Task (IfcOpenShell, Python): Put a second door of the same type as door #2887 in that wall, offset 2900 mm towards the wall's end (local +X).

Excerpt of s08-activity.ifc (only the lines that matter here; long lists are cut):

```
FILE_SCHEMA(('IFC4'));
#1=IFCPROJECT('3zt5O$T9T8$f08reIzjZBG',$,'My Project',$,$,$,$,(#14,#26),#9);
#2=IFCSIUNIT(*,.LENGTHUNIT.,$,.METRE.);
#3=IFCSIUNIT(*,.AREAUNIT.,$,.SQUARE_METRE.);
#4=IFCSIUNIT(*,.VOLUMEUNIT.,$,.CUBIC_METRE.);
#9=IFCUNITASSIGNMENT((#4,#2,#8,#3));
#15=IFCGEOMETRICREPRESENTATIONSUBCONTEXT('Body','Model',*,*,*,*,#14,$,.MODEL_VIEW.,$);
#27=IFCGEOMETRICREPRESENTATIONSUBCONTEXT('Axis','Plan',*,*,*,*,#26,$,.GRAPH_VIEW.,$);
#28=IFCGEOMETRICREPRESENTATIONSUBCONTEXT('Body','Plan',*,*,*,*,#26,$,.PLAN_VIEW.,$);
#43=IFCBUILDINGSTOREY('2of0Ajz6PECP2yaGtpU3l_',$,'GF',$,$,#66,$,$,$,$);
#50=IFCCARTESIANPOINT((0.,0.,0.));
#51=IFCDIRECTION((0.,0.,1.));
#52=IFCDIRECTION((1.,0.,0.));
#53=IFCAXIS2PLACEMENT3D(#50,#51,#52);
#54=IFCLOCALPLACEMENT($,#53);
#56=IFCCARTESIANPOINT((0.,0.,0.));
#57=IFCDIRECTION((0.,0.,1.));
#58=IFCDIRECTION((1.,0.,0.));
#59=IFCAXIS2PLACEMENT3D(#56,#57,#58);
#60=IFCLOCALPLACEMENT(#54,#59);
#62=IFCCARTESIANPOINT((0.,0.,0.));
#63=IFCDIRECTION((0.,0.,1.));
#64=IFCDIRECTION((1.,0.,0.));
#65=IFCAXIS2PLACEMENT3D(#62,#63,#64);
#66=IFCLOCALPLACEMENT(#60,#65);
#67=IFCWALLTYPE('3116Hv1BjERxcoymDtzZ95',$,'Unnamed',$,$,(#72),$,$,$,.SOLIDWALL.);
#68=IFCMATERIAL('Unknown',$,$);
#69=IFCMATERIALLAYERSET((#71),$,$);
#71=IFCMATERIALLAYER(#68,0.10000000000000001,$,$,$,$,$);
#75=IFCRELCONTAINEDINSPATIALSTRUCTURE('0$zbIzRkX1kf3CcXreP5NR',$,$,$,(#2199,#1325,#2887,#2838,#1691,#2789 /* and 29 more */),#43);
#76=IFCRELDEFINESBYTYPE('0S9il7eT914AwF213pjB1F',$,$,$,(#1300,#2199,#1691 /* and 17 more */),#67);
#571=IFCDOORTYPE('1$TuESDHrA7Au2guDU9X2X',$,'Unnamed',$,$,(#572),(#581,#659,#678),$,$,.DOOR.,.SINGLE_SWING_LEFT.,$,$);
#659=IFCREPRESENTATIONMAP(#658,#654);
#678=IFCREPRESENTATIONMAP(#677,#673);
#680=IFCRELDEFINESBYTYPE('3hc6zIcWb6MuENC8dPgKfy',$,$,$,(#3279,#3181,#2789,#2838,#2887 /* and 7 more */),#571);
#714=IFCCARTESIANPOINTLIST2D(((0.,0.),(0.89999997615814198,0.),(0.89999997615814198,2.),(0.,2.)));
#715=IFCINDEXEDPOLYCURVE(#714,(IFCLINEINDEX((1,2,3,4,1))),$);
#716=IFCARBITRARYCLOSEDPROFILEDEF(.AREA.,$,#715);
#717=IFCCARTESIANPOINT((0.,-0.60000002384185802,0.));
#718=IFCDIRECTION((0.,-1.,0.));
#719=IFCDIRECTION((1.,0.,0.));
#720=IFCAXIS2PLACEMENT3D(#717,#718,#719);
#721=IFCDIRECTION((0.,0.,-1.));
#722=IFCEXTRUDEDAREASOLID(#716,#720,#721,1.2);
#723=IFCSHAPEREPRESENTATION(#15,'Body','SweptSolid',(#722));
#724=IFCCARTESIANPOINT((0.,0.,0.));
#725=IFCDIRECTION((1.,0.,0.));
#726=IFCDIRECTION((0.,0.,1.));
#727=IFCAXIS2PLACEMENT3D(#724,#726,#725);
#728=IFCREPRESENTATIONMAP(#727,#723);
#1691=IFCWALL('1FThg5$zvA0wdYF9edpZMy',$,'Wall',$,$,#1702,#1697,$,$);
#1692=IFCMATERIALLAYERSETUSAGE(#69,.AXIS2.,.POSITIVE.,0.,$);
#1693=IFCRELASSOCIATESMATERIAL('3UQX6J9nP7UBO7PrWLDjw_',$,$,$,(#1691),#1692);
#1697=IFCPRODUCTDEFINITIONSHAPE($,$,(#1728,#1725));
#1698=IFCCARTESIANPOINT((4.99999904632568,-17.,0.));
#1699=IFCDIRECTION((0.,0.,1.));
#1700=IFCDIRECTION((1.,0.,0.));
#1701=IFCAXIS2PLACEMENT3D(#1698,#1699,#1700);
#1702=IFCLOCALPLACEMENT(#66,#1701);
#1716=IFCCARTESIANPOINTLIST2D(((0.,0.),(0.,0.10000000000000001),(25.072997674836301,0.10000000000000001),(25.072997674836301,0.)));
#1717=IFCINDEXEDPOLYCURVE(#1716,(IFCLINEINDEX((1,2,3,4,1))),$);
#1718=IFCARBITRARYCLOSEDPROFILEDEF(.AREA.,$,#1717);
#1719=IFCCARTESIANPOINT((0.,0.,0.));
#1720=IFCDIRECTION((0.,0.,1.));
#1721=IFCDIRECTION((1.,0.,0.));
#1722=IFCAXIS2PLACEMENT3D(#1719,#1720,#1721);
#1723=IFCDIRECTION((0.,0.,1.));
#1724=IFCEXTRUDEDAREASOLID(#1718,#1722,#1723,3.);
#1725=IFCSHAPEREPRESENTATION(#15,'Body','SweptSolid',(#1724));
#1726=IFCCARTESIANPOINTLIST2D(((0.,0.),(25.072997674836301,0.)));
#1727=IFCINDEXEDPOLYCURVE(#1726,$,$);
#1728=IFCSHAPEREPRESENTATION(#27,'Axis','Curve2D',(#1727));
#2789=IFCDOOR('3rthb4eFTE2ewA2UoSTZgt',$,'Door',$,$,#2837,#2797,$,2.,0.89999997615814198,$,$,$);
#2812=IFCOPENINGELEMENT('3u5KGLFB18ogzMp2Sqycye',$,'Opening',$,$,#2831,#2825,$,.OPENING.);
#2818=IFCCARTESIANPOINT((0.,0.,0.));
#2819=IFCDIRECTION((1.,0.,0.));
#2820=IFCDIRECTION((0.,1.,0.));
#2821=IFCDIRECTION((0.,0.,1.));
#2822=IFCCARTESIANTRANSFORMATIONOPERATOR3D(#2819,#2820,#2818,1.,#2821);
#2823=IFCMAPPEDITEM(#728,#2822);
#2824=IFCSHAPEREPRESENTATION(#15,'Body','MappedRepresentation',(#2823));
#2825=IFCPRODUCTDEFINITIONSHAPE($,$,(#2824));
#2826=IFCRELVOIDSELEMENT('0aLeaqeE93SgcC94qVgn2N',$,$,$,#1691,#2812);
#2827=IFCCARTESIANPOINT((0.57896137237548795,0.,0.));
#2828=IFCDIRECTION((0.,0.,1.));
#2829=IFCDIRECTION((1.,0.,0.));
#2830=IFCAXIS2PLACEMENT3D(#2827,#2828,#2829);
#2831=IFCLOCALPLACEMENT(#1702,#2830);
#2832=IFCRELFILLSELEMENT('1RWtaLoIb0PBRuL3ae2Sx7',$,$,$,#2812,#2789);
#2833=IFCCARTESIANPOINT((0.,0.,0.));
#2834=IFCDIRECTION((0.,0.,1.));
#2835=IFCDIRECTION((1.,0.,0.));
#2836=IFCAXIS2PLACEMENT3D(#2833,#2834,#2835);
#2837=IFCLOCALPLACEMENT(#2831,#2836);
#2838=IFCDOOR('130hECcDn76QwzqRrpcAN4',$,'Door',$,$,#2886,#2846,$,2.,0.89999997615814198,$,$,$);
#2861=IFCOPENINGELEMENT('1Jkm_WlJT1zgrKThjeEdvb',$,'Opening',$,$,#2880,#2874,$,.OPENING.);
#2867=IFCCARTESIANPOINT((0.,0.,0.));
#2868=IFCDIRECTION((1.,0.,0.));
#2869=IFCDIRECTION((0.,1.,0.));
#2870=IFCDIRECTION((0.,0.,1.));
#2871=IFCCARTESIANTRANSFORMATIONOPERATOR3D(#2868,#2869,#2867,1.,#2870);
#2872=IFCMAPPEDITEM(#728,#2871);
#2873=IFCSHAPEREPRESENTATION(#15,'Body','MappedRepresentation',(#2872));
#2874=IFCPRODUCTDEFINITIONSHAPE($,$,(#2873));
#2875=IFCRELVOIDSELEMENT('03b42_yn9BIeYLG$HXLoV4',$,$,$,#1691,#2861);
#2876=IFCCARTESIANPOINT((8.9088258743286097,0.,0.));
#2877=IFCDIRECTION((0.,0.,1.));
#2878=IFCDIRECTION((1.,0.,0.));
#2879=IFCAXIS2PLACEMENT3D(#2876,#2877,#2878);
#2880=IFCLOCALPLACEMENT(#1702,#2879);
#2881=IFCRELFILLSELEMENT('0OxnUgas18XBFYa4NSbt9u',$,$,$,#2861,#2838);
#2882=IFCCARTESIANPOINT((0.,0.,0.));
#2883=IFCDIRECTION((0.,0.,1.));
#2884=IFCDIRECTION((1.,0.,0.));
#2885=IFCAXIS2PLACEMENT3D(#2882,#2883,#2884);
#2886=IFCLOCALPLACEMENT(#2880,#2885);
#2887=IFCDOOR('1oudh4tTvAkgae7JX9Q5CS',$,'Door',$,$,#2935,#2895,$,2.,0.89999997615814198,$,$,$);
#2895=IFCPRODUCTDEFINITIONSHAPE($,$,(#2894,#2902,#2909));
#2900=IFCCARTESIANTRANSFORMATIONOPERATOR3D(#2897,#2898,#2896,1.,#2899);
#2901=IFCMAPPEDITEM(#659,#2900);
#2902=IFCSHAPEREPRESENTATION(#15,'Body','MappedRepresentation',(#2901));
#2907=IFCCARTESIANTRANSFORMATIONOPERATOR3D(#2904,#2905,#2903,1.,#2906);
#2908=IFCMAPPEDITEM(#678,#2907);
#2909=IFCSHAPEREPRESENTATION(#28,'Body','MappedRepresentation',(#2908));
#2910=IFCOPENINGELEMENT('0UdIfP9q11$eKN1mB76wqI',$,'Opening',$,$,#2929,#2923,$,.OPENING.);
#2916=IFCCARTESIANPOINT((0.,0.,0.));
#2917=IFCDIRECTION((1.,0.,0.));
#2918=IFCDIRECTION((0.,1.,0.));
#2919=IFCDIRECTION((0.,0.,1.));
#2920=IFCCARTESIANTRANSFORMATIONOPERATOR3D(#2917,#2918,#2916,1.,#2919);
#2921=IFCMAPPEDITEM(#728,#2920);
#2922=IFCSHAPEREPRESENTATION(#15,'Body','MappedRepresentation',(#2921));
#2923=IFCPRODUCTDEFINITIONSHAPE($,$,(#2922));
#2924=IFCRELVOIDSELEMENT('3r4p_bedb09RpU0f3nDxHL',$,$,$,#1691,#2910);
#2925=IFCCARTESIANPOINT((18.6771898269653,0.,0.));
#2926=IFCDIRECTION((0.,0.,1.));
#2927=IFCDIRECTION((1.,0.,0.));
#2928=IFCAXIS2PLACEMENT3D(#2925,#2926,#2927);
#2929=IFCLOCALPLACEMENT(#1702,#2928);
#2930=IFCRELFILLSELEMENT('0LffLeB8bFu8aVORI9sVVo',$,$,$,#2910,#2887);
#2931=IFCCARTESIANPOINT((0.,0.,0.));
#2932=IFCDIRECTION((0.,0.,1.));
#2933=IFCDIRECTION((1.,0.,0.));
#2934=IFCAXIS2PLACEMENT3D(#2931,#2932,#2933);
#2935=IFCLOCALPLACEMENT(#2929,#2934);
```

```python
import ifcopenshell
import ifcopenshell.api.feature
import ifcopenshell.api.geometry
import ifcopenshell.api.root
import ifcopenshell.geom
import ifcopenshell.util.element
import ifcopenshell.util.placement
import ifcopenshell.util.shape

model = ifcopenshell.open("s08-activity.ifc")
settings = ifcopenshell.geom.settings()


def volume(element):
    """Net volume in cubic metres, openings subtracted."""
    shape = ifcopenshell.geom.create_shape(settings, element)
    return ifcopenshell.util.shape.get_volume(shape.geometry)


door = model.by_guid("1oudh4tTvAkgae7JX9Q5CS")
opening = door.FillsVoids[0].RelatingOpeningElement
wall = opening.VoidsElements[0].RelatingBuildingElement
before = volume(wall)
shift = ifcopenshell.util.placement.get_local_placement(wall.ObjectPlacement)[:3, 0] * 2.9

# copy_class copies the void relationship, type, container and properties, but no geometry.
new_opening = ifcopenshell.api.root.copy_class(model, product=opening)
new_opening.Representation = ifcopenshell.util.element.copy_deep(
    model, opening.Representation, exclude=["IfcGeometricRepresentationContext", "IfcRepresentationMap"]
)
new_door = ifcopenshell.api.root.copy_class(model, product=door)
new_door.Representation = ifcopenshell.util.element.copy_deep(
    model, door.Representation, exclude=["IfcGeometricRepresentationContext", "IfcRepresentationMap"]
)
ifcopenshell.api.feature.add_filling(model, opening=new_opening, element=new_door)

for old, new in ((opening, new_opening), (door, new_door)):
    matrix = ifcopenshell.util.placement.get_local_placement(old.ObjectPlacement)
    matrix[:3, 3] += shift
    ifcopenshell.api.geometry.edit_object_placement(model, product=new, matrix=matrix, is_si=False)

after = volume(wall)

print(f"wall volume {before:.3f} -> {after:.3f} m3")

model.write("s08-activity_rev.ifc")
```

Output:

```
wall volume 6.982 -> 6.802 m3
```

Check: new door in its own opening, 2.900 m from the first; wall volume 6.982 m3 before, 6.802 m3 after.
